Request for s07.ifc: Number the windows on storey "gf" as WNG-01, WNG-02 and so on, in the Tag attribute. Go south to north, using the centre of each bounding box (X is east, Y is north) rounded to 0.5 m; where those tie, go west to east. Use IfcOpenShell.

First a look at what the model holds.

```python
import ifcopenshell
import ifcopenshell.util.element
import ifcopenshell.util.placement

model = ifcopenshell.open("s07.ifc")
print(model.schema)
storey = next(s for s in model.by_type("IfcBuildingStorey") if s.Name == "gf")
windows = [e for e in ifcopenshell.util.element.get_decomposition(storey) if e.is_a("IfcWindow")]
for e in sorted(windows, key=lambda e: e.id()):
    origin = ifcopenshell.util.placement.get_local_placement(e.ObjectPlacement)[:3, 3]
    print(e.id(), e.Tag, e.Name, origin.round(2) + 0.0, sep=" | ")
```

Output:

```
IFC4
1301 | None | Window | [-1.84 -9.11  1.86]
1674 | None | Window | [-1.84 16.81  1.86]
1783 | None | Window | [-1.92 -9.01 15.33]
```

```python
import ifcopenshell
import ifcopenshell.geom
import ifcopenshell.util.element
import ifcopenshell.util.shape

model = ifcopenshell.open("s07.ifc")
settings = ifcopenshell.geom.settings()
settings.set("use-world-coords", True)


def centre(element):
    shape = ifcopenshell.geom.create_shape(settings, element)
    return ifcopenshell.util.shape.get_bbox_centroid(shape.geometry)


storey = next(s for s in model.by_type("IfcBuildingStorey") if s.Name == "gf")
windows = [e for e in ifcopenshell.util.element.get_decomposition(storey) if e.is_a("IfcWindow")]

# Insertion points can sit at a corner or the storey origin, so sort by the geometry (in metres).
centres = {e: centre(e) for e in windows}
windows.sort(key=lambda e: (round(centres[e][1] / 0.5), centres[e][0]))

for i, e in enumerate(windows, start=1):
    number = f"WNG-{i:02d}"
    e.Tag = number
    print(e.id(), number)

model.write("s07_v2.ifc")
```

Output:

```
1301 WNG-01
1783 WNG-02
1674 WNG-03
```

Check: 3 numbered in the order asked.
